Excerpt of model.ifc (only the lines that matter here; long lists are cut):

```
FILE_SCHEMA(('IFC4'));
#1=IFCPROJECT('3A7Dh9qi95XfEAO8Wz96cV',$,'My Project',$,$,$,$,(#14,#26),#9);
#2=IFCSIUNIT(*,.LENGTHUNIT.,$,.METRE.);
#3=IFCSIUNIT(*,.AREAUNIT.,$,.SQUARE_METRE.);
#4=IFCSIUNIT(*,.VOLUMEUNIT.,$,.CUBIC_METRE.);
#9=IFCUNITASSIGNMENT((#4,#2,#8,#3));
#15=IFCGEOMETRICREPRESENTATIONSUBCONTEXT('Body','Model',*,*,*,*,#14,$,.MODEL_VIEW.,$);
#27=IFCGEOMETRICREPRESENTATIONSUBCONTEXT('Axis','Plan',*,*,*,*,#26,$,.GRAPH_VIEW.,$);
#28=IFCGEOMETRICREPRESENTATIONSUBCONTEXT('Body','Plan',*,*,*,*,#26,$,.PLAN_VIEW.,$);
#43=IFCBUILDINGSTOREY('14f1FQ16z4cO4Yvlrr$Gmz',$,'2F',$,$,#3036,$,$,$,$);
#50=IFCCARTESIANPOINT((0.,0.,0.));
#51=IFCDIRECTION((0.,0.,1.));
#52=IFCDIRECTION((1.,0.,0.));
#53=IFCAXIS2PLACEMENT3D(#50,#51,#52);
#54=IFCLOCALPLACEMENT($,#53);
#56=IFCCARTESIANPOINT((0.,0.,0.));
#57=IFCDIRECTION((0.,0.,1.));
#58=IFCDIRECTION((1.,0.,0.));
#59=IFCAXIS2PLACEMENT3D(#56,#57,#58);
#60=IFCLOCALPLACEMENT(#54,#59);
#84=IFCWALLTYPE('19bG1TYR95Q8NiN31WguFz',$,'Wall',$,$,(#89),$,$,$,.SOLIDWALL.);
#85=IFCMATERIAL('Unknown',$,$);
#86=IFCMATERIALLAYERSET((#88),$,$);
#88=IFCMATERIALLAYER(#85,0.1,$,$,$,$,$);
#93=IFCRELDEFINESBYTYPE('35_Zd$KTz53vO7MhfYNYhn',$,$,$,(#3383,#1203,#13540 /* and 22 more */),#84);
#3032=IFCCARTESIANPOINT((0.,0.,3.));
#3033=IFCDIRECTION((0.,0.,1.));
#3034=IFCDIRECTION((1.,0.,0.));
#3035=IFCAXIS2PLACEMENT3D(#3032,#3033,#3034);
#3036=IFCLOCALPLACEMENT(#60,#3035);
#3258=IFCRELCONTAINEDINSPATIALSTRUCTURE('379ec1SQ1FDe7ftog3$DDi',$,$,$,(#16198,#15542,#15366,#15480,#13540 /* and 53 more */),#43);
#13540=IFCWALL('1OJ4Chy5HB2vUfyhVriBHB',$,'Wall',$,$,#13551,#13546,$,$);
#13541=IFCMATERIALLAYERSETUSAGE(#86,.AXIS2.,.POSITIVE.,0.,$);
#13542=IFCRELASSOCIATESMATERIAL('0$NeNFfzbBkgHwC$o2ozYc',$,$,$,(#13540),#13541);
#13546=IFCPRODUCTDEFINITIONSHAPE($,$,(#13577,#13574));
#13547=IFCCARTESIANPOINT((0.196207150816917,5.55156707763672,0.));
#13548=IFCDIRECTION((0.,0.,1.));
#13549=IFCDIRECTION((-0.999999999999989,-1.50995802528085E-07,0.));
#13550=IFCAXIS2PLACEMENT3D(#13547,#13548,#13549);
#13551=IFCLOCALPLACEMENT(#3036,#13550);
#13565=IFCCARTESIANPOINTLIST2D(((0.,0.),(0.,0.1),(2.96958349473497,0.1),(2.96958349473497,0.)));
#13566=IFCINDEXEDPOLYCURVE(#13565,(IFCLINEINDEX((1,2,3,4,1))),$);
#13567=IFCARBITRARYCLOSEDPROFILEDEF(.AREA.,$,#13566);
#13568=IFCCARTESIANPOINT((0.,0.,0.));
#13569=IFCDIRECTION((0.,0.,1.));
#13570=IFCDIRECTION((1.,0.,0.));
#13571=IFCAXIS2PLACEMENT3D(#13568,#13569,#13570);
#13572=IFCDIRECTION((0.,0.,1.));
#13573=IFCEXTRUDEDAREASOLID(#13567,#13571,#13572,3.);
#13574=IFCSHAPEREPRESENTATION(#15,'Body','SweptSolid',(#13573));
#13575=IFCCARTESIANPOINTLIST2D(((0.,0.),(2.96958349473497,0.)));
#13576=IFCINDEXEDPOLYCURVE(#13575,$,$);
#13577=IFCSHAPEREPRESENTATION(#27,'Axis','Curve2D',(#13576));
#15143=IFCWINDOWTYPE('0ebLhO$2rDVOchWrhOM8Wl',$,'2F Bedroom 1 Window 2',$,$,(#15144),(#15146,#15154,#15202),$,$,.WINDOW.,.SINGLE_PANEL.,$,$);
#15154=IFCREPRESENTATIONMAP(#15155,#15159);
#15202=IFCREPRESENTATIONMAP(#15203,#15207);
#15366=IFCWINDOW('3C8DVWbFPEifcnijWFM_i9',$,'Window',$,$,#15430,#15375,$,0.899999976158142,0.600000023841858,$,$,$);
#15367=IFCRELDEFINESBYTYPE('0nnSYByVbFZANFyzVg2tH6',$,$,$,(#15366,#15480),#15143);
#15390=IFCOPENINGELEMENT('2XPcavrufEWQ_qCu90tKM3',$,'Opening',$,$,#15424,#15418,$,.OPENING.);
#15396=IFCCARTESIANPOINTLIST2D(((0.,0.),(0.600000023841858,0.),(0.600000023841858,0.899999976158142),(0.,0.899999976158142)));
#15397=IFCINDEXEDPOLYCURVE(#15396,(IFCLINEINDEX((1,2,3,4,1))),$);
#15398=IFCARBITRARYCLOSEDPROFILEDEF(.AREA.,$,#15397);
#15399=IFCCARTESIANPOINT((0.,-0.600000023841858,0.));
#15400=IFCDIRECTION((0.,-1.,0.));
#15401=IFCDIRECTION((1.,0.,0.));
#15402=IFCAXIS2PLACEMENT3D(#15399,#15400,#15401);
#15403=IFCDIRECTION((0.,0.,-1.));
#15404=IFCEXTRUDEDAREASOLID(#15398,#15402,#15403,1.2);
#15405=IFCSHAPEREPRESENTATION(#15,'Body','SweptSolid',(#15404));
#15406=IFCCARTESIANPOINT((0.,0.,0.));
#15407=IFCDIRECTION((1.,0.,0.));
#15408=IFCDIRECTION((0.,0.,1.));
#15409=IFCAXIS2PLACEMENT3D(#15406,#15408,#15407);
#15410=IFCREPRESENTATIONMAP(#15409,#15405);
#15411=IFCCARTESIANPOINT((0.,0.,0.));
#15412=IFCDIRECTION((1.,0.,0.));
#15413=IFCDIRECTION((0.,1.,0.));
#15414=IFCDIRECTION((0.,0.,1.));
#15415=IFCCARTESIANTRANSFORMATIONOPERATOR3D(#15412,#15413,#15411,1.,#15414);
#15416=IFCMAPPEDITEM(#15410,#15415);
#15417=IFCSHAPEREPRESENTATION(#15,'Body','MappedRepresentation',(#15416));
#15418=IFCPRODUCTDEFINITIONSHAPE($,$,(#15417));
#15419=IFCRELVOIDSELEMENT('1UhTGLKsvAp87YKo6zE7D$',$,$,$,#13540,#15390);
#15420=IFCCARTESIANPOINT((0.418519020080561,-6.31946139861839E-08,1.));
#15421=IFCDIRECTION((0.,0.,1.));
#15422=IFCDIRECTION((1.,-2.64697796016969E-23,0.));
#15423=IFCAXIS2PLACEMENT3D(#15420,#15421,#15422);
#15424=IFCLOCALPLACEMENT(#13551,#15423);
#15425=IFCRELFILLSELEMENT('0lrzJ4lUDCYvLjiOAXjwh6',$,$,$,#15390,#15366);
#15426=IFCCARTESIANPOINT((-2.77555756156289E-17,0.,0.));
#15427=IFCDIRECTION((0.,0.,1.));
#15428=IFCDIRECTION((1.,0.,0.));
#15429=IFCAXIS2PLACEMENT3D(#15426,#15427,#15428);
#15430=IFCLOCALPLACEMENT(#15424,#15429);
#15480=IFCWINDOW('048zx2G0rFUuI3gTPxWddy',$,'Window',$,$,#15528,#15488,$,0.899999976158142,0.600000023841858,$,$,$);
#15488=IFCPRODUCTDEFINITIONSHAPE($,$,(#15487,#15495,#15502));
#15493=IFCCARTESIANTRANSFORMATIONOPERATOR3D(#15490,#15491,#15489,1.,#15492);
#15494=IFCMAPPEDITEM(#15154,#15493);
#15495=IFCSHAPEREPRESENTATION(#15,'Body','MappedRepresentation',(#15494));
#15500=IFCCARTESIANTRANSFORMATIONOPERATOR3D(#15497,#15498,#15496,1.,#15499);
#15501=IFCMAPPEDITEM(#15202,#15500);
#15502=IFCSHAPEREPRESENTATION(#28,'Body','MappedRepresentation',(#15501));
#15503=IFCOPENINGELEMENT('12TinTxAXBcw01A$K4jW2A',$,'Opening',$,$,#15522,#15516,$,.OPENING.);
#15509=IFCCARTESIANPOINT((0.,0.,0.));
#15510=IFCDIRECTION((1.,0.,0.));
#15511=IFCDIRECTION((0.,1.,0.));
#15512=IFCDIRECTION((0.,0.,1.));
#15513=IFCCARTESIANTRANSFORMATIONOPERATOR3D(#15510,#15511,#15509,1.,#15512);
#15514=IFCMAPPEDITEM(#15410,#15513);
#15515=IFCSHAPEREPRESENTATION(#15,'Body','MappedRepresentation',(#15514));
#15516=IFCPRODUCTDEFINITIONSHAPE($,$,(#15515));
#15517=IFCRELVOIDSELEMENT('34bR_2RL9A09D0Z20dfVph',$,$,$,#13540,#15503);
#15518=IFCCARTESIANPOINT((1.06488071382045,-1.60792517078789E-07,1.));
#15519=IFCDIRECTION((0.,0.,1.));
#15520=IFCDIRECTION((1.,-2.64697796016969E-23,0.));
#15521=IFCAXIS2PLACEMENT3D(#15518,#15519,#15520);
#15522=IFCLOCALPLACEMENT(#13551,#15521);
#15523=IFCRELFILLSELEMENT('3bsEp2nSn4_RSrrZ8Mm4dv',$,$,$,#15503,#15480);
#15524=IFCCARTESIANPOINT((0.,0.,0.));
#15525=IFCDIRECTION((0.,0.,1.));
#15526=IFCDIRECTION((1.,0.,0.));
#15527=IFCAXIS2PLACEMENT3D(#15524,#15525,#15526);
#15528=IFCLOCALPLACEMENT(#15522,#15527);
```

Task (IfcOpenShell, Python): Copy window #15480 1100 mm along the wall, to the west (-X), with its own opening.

```python
import ifcopenshell
import ifcopenshell.api.feature
import ifcopenshell.api.geometry
import ifcopenshell.api.root
import ifcopenshell.geom
import ifcopenshell.util.element
import ifcopenshell.util.placement
import ifcopenshell.util.shape

model = ifcopenshell.open("model.ifc")
settings = ifcopenshell.geom.settings()


def volume(element):
    """Net volume in cubic metres, openings subtracted."""
    shape = ifcopenshell.geom.create_shape(settings, element)
    return ifcopenshell.util.shape.get_volume(shape.geometry)


window = model.by_guid("048zx2G0rFUuI3gTPxWddy")
opening = window.FillsVoids[0].RelatingOpeningElement
wall = opening.VoidsElements[0].RelatingBuildingElement
before = volume(wall)
shift = ifcopenshell.util.placement.get_local_placement(wall.ObjectPlacement)[:3, 0] * 1.1

# copy_class copies the void relationship, type, container and properties, but no geometry.
new_opening = ifcopenshell.api.root.copy_class(model, product=opening)
new_opening.Representation = ifcopenshell.util.element.copy_deep(
    model, opening.Representation, exclude=["IfcGeometricRepresentationContext", "IfcRepresentationMap"]
)
new_window = ifcopenshell.api.root.copy_class(model, product=window)
new_window.Representation = ifcopenshell.util.element.copy_deep(
    model, window.Representation, exclude=["IfcGeometricRepresentationContext", "IfcRepresentationMap"]
)
ifcopenshell.api.feature.add_filling(model, opening=new_opening, element=new_window)

for old, new in ((opening, new_opening), (window, new_window)):
    matrix = ifcopenshell.util.placement.get_local_placement(old.ObjectPlacement)
    matrix[:3, 3] += shift
    ifcopenshell.api.geometry.edit_object_placement(model, product=new, matrix=matrix, is_si=False)

after = volume(wall)

print(f"wall volume {before:.3f} -> {after:.3f} m3")

model.write("model_edited.ifc")
```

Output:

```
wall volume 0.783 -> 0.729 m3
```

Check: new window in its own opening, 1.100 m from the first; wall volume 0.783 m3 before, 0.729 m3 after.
